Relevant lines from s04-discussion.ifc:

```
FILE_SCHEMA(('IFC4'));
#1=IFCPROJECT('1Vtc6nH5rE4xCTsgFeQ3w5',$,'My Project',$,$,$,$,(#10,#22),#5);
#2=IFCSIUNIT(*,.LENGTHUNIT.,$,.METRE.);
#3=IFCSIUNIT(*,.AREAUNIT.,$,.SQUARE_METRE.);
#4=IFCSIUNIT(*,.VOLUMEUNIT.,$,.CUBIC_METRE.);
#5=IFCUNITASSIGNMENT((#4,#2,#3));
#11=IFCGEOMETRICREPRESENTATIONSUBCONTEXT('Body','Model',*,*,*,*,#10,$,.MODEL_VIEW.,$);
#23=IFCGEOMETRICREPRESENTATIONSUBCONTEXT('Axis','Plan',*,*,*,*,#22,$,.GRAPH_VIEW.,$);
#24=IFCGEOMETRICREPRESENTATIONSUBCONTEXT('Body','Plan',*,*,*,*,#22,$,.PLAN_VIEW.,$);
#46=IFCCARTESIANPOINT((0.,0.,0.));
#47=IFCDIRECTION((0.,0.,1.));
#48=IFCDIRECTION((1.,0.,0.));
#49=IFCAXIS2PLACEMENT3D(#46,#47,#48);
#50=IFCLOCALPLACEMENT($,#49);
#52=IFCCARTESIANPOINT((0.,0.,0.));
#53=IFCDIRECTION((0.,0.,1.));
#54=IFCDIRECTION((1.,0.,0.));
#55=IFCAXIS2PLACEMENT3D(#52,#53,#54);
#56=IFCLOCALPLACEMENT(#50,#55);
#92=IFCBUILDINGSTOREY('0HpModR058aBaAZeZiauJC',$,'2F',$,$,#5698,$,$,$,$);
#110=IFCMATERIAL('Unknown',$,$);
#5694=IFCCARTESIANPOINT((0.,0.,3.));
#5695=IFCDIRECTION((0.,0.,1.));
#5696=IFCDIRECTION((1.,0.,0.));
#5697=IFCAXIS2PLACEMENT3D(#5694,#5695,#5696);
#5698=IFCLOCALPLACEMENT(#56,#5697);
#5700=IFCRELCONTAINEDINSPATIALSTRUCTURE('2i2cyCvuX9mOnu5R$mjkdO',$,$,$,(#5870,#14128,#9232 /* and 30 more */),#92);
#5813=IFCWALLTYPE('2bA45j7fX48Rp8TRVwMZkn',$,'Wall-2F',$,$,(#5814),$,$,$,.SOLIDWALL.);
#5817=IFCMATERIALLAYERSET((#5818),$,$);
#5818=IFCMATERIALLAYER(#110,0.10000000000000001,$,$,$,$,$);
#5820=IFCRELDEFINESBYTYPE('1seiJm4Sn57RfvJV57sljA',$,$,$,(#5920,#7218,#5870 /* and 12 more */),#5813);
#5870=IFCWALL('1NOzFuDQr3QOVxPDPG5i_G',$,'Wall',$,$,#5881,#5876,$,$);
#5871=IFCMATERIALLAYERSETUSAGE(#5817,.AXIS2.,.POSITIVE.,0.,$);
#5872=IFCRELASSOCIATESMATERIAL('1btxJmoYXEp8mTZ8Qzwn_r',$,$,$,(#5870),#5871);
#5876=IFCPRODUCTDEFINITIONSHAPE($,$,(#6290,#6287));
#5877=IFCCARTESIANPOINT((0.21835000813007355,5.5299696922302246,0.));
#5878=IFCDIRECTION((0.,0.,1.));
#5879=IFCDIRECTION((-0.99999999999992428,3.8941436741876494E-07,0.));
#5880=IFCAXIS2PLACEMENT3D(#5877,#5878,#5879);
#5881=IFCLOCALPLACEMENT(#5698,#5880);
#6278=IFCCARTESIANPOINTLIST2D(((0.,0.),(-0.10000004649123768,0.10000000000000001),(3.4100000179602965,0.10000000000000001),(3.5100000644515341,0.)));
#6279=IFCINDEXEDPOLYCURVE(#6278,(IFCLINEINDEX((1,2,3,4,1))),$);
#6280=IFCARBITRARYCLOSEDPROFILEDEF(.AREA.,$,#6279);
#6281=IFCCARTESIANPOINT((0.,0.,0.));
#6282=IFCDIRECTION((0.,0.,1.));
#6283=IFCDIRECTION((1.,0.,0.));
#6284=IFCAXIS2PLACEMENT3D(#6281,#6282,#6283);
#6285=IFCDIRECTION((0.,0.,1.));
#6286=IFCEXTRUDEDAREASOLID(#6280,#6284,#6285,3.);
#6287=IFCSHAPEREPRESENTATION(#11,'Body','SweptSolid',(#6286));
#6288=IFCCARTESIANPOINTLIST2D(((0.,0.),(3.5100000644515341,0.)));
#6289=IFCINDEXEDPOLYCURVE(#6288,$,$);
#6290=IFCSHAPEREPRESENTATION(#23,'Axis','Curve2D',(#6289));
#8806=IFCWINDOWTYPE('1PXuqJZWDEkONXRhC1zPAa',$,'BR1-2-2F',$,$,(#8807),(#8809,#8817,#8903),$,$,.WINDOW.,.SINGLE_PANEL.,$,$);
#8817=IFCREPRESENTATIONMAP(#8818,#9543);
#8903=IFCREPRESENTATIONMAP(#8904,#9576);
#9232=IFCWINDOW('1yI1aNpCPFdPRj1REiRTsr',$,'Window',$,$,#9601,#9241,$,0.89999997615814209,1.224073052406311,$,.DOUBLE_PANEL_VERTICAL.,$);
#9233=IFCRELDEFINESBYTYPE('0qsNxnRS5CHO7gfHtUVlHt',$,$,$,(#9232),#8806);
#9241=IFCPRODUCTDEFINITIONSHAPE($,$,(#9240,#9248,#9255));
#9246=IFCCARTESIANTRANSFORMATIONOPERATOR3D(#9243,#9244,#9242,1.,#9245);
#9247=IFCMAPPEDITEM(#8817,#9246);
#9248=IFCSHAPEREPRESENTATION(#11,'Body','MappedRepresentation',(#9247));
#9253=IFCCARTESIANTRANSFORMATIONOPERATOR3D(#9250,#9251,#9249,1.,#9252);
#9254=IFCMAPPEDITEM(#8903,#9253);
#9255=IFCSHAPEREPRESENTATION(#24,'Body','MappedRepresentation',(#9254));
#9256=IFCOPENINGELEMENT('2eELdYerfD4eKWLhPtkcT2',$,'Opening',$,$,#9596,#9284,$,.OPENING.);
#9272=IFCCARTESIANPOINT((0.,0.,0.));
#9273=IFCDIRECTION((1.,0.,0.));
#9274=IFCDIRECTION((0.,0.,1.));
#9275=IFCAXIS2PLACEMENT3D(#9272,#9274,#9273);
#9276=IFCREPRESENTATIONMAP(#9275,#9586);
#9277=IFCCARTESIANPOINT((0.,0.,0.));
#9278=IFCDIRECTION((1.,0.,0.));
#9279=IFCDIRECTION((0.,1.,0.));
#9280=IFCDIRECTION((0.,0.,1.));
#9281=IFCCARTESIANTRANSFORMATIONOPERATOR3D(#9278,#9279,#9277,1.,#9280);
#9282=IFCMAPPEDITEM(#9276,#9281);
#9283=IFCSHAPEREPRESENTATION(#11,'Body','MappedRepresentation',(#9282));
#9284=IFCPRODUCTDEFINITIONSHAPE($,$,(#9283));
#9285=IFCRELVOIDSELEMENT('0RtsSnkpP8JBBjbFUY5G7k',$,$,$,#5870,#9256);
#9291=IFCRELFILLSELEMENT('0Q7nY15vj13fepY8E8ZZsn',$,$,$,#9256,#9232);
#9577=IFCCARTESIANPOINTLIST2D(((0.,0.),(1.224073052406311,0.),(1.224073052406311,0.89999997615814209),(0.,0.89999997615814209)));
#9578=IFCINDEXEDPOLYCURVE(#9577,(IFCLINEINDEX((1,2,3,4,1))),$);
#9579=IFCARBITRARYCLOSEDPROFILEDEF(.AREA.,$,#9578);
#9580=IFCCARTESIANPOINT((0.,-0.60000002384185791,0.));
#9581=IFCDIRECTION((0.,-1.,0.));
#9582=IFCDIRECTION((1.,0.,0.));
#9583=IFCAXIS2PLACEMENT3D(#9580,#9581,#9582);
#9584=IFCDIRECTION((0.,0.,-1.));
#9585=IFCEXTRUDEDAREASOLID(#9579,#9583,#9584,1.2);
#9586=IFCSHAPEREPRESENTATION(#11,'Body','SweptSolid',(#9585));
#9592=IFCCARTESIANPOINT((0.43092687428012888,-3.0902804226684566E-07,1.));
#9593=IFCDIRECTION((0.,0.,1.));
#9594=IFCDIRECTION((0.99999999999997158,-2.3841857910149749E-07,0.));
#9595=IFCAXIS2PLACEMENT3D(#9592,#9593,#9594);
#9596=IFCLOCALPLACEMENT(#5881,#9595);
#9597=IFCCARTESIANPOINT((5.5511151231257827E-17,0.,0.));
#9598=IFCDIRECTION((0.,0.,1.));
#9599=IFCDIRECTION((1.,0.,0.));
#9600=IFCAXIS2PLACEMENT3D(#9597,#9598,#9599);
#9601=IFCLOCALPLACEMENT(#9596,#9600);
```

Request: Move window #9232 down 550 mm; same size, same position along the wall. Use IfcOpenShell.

```python
import numpy as np
import ifcopenshell
import ifcopenshell.api.geometry
import ifcopenshell.util.placement
import ifcopenshell.util.unit

model = ifcopenshell.open("s04-discussion.ifc")
unit_scale = ifcopenshell.util.unit.calculate_unit_scale(model)

window = model.by_id(9232)
opening = window.FillsVoids[0].RelatingOpeningElement
dz = -0.55 / unit_scale

shift = np.array([0.0, 0.0, dz])
# The window is placed relative to its opening, so it follows when the opening moves.
matrix = ifcopenshell.util.placement.get_local_placement(opening.ObjectPlacement)
matrix[:3, 3] += shift
ifcopenshell.api.geometry.edit_object_placement(
    model, product=opening, matrix=matrix, is_si=False, should_transform_children=True
)

print(f"moved by {dz * unit_scale:+.3f} m")

model.write("s04-discussion_updated.ifc")
```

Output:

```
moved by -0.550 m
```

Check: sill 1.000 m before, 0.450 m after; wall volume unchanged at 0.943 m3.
